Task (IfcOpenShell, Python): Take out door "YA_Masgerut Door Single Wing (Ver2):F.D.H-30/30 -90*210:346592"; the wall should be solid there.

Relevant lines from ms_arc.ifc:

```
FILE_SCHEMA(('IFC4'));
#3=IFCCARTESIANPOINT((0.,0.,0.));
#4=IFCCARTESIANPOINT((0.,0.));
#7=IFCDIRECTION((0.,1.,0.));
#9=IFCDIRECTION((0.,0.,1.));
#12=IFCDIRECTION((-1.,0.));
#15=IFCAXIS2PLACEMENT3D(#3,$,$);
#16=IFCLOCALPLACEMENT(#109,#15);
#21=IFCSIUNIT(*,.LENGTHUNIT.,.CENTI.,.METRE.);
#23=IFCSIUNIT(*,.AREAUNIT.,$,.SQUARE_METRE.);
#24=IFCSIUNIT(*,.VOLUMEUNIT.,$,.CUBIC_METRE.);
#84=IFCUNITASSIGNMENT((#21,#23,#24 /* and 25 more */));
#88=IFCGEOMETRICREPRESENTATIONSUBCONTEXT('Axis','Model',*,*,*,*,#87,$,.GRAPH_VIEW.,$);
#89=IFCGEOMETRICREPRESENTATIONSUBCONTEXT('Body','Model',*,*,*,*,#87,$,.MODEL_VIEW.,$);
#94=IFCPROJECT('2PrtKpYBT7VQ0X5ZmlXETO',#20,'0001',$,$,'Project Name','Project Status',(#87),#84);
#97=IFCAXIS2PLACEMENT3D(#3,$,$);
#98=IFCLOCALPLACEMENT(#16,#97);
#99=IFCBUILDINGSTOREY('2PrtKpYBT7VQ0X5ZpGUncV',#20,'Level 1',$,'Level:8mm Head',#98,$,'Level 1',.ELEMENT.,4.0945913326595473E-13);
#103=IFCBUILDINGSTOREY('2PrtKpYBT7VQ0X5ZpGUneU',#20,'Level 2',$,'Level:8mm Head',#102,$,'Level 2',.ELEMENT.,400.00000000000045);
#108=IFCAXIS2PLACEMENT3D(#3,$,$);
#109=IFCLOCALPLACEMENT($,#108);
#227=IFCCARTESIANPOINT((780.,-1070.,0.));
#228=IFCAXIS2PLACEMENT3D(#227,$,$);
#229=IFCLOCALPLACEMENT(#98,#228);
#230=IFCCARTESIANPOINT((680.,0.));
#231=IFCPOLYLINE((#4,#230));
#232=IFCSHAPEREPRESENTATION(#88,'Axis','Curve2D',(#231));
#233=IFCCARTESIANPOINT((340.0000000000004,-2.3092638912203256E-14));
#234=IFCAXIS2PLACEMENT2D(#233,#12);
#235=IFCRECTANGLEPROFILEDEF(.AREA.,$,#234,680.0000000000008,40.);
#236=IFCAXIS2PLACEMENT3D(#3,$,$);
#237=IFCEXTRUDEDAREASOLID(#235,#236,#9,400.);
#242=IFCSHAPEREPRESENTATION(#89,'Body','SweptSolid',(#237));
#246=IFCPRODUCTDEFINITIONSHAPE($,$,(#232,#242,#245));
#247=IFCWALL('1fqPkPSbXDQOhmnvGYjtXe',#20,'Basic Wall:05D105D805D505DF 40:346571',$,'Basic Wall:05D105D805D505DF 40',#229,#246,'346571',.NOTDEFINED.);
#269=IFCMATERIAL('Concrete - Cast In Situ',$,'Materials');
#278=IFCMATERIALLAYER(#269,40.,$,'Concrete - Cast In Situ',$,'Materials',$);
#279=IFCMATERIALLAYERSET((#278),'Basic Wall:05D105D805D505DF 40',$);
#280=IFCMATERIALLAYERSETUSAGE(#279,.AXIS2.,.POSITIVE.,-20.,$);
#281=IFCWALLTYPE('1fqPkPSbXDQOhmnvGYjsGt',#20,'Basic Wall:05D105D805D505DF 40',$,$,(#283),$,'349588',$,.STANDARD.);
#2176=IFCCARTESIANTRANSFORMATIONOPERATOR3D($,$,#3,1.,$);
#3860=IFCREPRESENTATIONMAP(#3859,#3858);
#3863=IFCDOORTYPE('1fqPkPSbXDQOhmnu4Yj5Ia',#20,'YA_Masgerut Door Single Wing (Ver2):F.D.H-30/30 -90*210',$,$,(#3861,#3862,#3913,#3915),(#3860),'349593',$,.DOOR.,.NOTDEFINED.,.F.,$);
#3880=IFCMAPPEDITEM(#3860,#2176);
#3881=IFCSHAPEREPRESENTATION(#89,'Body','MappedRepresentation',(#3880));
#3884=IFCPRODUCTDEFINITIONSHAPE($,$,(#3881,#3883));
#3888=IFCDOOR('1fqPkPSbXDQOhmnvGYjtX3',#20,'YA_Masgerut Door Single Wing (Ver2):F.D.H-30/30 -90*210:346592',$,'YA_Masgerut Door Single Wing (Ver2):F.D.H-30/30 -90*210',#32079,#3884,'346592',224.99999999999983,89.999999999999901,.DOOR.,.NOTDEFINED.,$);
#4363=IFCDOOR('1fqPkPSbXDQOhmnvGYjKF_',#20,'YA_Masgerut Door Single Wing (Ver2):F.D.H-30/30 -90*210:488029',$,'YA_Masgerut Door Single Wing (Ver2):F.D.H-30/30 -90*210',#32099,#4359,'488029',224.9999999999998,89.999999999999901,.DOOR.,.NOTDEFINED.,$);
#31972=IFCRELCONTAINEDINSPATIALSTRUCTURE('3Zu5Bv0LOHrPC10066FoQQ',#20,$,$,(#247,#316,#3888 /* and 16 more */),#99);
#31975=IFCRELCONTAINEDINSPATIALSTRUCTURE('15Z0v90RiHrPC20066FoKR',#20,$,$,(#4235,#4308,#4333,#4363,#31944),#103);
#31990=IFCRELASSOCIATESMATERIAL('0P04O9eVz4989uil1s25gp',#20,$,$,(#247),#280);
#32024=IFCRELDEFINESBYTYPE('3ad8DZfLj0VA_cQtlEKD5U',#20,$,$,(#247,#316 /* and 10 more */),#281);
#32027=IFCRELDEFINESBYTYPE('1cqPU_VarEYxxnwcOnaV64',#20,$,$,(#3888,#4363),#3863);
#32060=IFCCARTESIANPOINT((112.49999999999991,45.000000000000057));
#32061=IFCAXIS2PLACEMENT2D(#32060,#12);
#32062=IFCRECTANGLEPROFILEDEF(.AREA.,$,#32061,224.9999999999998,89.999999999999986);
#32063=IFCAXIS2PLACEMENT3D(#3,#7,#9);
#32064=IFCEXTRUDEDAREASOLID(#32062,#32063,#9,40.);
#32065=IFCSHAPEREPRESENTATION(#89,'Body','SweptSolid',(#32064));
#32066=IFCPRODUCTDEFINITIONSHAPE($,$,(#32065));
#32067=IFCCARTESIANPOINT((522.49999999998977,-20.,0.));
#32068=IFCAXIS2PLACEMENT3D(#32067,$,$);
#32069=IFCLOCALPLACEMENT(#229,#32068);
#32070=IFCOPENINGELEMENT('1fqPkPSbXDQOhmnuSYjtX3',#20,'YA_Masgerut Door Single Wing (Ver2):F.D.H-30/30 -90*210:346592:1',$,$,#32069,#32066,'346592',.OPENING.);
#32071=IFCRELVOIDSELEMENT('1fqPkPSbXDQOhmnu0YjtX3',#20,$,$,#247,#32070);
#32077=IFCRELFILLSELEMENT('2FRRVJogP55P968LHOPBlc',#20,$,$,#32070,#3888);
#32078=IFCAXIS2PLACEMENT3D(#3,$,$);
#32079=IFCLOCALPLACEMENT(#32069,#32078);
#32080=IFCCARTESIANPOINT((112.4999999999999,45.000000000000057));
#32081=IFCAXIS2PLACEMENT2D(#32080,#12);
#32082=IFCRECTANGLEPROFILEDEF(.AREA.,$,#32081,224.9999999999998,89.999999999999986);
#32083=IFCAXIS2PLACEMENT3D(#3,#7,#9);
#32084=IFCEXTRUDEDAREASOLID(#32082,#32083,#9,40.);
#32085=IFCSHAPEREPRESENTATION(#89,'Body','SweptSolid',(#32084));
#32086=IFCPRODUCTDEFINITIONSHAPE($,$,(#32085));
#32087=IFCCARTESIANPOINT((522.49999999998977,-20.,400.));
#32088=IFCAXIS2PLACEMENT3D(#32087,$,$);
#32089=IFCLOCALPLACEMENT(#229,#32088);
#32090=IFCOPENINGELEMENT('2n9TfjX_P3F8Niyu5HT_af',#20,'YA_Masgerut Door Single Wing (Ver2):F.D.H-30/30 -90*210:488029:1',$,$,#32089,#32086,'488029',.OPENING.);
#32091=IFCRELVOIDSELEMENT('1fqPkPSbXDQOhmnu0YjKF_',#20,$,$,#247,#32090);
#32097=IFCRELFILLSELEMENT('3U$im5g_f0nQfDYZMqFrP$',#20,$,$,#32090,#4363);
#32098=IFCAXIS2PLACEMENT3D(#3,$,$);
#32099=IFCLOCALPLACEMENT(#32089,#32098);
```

```python
import ifcopenshell
import ifcopenshell.api.feature
import ifcopenshell.api.root
import ifcopenshell.geom
import ifcopenshell.util.shape

model = ifcopenshell.open("ms_arc.ifc")
settings = ifcopenshell.geom.settings()


def volume(element):
    """Net volume in cubic metres, openings subtracted."""
    shape = ifcopenshell.geom.create_shape(settings, element)
    return ifcopenshell.util.shape.get_volume(shape.geometry)


door = model.by_id(3888)
opening = door.FillsVoids[0].RelatingOpeningElement
wall = opening.VoidsElements[0].RelatingBuildingElement
before = volume(wall)

ifcopenshell.api.root.remove_product(model, product=door)
ifcopenshell.api.feature.remove_feature(model, feature=opening)

after = volume(wall)

print(f"wall volume {before:.3f} -> {after:.3f} m3")

model.write("ms_arc_rev.ifc")
```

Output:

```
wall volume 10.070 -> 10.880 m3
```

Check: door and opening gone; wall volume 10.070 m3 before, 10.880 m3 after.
